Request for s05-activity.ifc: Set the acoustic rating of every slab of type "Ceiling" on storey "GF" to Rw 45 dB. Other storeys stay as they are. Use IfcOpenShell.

First a look at what the model holds.

```python
import ifcopenshell
import ifcopenshell.util.element

model = ifcopenshell.open("s05-activity.ifc")
print(model.schema)
storey = next(s for s in model.by_type("IfcBuildingStorey") if s.Name == "GF")
slabs = [e for e in ifcopenshell.util.element.get_decomposition(storey) if e.is_a("IfcSlab")]
seen = {}
for e in slabs:
    element_type = ifcopenshell.util.element.get_type(e)
    key = (element_type.Name if element_type != e and element_type else None, ifcopenshell.util.element.get_pset(e, "Pset_SlabCommon", "AcousticRating"))
    seen[key] = seen.get(key, 0) + 1
for (name, value), count in sorted(seen.items(), key=str):
    print(count, "x", name, "|", value)
```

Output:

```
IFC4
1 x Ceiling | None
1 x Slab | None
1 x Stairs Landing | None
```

```python
import ifcopenshell
import ifcopenshell.api.pset
import ifcopenshell.util.element

model = ifcopenshell.open("s05-activity.ifc")

storey = next(s for s in model.by_type("IfcBuildingStorey") if s.Name == "GF")
slabs = [e for e in ifcopenshell.util.element.get_decomposition(storey) if e.is_a("IfcSlab")]

count = 0
for e in slabs:
    element_type = ifcopenshell.util.element.get_type(e)
    if element_type in (None, e) or element_type.Name != "Ceiling":
        continue
    # add_pset returns the element's existing set when there is one.
    pset = ifcopenshell.api.pset.add_pset(model, product=e, name="Pset_SlabCommon")
    ifcopenshell.api.pset.edit_pset(model, pset=pset, properties={"AcousticRating": "Rw 45 dB"})
    count += 1

print(count, "slabs updated")

model.write("s05-activity_rev.ifc")
```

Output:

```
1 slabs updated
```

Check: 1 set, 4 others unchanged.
